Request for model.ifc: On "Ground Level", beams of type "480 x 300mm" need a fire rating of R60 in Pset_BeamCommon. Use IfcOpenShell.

First a look at what the model holds.

```python
import ifcopenshell
import ifcopenshell.util.element

model = ifcopenshell.open("model.ifc")
print(model.schema)
storey = next(s for s in model.by_type("IfcBuildingStorey") if s.Name == "Ground Level")
beams = [e for e in ifcopenshell.util.element.get_decomposition(storey) if e.is_a("IfcBeam")]
seen = {}
for e in beams:
    element_type = ifcopenshell.util.element.get_type(e)
    key = (element_type.Name if element_type != e and element_type else None, ifcopenshell.util.element.get_pset(e, "Pset_BeamCommon", "FireRating"))
    seen[key] = seen.get(key, 0) + 1
for (name, value), count in sorted(seen.items(), key=str):
    print(count, "x", name, "|", value)
```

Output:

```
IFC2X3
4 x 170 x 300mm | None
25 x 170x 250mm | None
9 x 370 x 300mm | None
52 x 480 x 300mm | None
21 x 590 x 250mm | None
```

```python
import ifcopenshell
import ifcopenshell.api.pset
import ifcopenshell.util.element

model = ifcopenshell.open("model.ifc")

storey = next(s for s in model.by_type("IfcBuildingStorey") if s.Name == "Ground Level")
beams = [e for e in ifcopenshell.util.element.get_decomposition(storey) if e.is_a("IfcBeam")]

count = 0
for e in beams:
    element_type = ifcopenshell.util.element.get_type(e)
    if element_type in (None, e) or element_type.Name != "480 x 300mm":
        continue
    # add_pset returns the element's existing set when there is one.
    pset = ifcopenshell.api.pset.add_pset(model, product=e, name="Pset_BeamCommon")
    ifcopenshell.api.pset.edit_pset(model, pset=pset, properties={"FireRating": "R60"})
    count += 1

print(count, "beams updated")

model.write("model_rev.ifc")
```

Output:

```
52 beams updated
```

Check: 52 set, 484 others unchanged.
